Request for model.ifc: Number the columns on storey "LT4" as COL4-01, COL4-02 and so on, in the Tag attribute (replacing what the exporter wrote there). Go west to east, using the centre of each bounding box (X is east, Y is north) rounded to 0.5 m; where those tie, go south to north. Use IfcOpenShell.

First a look at what the model holds.

```python
import ifcopenshell
import ifcopenshell.util.element
import ifcopenshell.util.placement

model = ifcopenshell.open("model.ifc")
print(model.schema)
storey = next(s for s in model.by_type("IfcBuildingStorey") if s.Name == "LT4")
columns = [e for e in ifcopenshell.util.element.get_decomposition(storey) if e.is_a("IfcColumn")]
for e in sorted(columns, key=lambda e: e.id()):
    origin = ifcopenshell.util.placement.get_local_placement(e.ObjectPlacement)[:3, 3]
    print(e.id(), e.Tag, e.Name, origin.round(2) + 0.0, sep=" | ")
```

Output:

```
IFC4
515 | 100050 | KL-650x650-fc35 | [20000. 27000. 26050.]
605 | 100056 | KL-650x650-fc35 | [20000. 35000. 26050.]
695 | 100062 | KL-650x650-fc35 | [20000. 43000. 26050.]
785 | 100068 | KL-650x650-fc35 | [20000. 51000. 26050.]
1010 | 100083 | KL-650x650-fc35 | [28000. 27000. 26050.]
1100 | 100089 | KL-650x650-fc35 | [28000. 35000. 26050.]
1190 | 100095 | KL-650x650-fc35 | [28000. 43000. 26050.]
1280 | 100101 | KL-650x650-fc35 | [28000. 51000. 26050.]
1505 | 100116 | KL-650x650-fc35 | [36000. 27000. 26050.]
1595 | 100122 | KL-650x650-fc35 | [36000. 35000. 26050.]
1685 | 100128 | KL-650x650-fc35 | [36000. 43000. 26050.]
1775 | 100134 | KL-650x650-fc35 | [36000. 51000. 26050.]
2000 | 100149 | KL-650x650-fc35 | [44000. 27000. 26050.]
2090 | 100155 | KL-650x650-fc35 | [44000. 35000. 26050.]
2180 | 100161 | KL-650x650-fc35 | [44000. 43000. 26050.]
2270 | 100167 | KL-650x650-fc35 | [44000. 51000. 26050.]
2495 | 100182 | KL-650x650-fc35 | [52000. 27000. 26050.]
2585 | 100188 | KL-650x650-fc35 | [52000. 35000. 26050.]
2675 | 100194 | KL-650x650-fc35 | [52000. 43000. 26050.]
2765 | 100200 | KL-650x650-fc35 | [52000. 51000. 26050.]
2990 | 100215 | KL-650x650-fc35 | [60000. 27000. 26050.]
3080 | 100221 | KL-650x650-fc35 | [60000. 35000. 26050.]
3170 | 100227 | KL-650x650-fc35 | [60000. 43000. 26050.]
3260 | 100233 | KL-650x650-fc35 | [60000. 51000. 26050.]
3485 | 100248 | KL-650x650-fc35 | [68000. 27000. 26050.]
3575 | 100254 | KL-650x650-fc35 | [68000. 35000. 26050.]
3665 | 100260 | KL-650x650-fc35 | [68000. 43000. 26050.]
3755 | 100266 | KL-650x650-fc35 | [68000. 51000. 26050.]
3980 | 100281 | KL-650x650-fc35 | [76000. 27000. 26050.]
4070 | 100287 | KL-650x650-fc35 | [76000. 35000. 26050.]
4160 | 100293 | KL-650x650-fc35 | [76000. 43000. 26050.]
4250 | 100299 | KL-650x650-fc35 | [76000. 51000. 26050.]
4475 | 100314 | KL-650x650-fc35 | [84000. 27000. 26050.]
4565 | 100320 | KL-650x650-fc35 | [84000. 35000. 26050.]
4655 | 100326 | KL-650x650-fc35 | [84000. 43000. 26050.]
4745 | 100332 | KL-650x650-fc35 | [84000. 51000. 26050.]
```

```python
import ifcopenshell
import ifcopenshell.geom
import ifcopenshell.util.element
import ifcopenshell.util.shape

model = ifcopenshell.open("model.ifc")
settings = ifcopenshell.geom.settings()
settings.set("use-world-coords", True)


def centre(element):
    shape = ifcopenshell.geom.create_shape(settings, element)
    return ifcopenshell.util.shape.get_bbox_centroid(shape.geometry)


storey = next(s for s in model.by_type("IfcBuildingStorey") if s.Name == "LT4")
columns = [e for e in ifcopenshell.util.element.get_decomposition(storey) if e.is_a("IfcColumn")]

# Insertion points can sit at a corner or the storey origin, so sort by the geometry (in metres).
centres = {e: centre(e) for e in columns}
columns.sort(key=lambda e: (round(centres[e][0] / 0.5), centres[e][1]))

for i, e in enumerate(columns, start=1):
    number = f"COL4-{i:02d}"
    e.Tag = number
    print(e.id(), number)

model.write("model_v2.ifc")
```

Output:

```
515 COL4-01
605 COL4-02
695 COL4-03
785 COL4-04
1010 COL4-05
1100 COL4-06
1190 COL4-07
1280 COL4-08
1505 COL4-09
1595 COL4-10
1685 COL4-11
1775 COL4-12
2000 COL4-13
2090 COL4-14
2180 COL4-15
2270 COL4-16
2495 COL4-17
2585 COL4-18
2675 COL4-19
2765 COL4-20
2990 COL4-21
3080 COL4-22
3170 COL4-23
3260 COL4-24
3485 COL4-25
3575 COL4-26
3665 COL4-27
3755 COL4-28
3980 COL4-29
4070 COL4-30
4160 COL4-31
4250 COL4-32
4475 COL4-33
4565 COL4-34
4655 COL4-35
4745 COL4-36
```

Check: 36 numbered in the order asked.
